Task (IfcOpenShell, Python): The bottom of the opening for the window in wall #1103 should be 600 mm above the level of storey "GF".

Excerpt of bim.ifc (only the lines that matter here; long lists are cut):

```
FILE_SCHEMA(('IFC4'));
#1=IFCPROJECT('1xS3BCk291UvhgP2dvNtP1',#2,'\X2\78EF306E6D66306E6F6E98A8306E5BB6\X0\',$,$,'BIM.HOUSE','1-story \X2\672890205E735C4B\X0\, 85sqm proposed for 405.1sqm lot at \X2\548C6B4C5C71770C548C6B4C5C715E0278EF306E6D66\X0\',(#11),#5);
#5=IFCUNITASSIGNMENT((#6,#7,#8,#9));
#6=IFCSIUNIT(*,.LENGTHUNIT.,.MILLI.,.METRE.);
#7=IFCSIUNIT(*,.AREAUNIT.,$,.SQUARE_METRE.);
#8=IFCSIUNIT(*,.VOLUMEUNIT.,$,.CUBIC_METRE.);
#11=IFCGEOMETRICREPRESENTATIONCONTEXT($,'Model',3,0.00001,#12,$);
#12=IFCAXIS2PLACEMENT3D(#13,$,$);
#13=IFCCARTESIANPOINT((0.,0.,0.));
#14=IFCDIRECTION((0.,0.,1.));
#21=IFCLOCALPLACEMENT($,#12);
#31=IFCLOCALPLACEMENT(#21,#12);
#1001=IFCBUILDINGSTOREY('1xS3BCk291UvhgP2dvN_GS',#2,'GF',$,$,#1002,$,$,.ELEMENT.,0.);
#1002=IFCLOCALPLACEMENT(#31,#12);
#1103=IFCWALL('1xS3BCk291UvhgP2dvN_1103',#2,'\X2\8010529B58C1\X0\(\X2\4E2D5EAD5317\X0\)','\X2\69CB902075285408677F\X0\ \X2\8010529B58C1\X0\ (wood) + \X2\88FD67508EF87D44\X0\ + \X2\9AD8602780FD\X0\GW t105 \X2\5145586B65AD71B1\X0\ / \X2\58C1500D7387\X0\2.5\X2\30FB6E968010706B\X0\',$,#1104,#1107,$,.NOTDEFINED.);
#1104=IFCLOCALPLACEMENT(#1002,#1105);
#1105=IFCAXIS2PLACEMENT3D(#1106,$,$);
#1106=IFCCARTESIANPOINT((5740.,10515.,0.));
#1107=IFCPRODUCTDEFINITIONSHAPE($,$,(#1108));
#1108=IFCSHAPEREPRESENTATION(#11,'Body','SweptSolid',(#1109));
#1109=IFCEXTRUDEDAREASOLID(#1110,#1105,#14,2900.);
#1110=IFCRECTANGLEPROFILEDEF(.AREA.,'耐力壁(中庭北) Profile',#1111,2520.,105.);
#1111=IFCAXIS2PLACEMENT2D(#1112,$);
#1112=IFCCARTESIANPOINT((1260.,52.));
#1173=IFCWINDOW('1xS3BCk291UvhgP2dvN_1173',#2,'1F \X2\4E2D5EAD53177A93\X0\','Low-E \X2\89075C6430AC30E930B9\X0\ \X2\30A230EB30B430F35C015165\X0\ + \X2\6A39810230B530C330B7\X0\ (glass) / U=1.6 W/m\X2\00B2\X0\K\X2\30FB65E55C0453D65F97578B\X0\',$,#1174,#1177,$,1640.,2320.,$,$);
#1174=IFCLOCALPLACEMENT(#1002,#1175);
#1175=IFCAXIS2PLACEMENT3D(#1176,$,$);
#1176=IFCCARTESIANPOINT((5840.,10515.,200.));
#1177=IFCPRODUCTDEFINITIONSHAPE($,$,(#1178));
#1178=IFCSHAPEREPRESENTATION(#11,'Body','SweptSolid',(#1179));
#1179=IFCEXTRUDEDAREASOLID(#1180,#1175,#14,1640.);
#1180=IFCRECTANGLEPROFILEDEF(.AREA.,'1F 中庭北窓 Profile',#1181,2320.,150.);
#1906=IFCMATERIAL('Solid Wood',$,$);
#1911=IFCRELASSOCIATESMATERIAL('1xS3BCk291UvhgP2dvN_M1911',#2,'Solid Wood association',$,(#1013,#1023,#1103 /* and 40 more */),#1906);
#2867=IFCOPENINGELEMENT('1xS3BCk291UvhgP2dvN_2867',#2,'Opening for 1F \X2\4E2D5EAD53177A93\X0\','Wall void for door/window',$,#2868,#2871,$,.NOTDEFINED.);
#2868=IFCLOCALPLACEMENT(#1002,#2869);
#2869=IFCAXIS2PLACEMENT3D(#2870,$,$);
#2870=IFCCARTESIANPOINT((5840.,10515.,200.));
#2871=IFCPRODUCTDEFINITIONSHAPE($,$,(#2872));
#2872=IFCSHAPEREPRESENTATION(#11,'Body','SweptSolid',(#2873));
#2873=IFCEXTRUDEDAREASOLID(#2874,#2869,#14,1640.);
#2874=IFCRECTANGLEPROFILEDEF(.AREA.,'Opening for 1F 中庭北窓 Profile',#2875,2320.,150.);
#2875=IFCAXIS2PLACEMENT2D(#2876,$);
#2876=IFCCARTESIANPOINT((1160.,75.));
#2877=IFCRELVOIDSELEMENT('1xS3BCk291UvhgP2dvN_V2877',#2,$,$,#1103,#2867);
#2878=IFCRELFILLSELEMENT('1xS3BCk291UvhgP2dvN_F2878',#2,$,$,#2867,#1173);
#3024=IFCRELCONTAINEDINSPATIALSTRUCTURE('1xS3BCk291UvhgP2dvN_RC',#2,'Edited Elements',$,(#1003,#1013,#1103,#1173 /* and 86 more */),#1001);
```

```python
import numpy as np
import ifcopenshell
import ifcopenshell.api.geometry
import ifcopenshell.geom
import ifcopenshell.util.element
import ifcopenshell.util.placement
import ifcopenshell.util.shape
import ifcopenshell.util.unit

model = ifcopenshell.open("bim.ifc")
unit_scale = ifcopenshell.util.unit.calculate_unit_scale(model)

window = model.by_id(1173)
opening = window.FillsVoids[0].RelatingOpeningElement
storey = ifcopenshell.util.element.get_container(window, ifc_class="IfcBuildingStorey")
level = ifcopenshell.util.placement.get_local_placement(storey.ObjectPlacement)[2, 3]

# The opening's origin need not be at the sill, so measure its lowest point.
shape = ifcopenshell.geom.create_shape(ifcopenshell.geom.settings(), opening)
bottom = ifcopenshell.util.shape.get_shape_bottom_elevation(shape, shape.geometry) / unit_scale
dz = level + 0.6 / unit_scale - bottom

shift = np.array([0.0, 0.0, dz])
# The window is not placed relative to its opening, so move both.
for product in (opening, window):
    matrix = ifcopenshell.util.placement.get_local_placement(product.ObjectPlacement)
    matrix[:3, 3] += shift
    ifcopenshell.api.geometry.edit_object_placement(model, product=product, matrix=matrix, is_si=False)

print(f"moved by {dz * unit_scale:+.3f} m")

model.write("bim_rev.ifc")
```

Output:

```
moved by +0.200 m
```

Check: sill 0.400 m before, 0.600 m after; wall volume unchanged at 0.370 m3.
